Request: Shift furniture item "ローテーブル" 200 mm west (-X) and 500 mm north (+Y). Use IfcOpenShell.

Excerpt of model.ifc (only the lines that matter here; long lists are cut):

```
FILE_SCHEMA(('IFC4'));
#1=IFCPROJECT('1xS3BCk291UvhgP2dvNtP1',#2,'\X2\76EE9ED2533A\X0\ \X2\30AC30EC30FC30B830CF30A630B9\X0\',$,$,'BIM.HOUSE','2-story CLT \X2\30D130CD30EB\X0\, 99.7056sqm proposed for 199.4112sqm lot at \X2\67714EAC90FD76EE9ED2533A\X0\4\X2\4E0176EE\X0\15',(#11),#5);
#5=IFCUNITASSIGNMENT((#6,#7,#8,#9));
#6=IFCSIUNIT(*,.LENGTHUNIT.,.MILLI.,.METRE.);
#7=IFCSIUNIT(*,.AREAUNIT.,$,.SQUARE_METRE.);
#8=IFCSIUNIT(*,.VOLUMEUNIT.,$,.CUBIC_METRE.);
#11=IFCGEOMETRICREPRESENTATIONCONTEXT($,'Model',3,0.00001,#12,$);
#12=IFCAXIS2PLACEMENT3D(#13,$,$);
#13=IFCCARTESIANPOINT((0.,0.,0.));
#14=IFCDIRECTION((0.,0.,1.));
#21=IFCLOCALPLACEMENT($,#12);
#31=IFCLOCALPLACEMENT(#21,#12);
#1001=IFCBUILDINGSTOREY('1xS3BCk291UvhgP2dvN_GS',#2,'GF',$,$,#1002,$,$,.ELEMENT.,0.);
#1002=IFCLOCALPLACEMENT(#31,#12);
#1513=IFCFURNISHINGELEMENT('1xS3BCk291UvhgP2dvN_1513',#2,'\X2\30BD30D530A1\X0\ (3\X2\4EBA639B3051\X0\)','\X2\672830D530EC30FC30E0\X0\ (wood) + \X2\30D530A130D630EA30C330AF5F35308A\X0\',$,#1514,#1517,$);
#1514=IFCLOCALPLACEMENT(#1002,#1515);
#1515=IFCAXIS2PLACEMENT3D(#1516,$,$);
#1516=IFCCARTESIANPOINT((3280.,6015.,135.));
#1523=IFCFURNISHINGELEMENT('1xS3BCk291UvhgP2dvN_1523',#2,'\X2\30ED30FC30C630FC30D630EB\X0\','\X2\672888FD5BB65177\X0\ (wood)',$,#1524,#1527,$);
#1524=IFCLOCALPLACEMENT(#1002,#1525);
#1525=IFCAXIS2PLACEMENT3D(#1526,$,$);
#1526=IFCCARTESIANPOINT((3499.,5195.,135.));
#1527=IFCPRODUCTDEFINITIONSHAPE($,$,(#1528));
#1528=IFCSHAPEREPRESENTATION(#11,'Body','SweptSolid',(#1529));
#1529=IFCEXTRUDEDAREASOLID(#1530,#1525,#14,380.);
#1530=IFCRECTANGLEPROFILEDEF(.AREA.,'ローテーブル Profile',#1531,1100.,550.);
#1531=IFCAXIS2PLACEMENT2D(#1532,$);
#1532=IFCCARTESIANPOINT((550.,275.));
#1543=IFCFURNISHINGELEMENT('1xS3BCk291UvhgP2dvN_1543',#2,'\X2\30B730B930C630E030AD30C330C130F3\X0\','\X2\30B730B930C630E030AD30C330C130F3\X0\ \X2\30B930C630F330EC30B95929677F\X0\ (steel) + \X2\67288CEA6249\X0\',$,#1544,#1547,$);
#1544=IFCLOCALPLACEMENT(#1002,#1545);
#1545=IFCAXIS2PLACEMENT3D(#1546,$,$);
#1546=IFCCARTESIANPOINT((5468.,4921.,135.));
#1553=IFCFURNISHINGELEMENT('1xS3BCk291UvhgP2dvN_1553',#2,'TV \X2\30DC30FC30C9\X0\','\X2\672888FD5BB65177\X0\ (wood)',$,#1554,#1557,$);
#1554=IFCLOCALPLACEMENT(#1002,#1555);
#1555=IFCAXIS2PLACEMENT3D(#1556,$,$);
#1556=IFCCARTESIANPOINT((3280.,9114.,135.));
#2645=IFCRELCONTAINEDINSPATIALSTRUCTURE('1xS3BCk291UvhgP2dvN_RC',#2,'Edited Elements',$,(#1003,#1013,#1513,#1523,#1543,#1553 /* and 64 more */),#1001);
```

```python
import ifcopenshell
import ifcopenshell.api.geometry
import ifcopenshell.util.placement
import ifcopenshell.util.unit

model = ifcopenshell.open("model.ifc")
unit_scale = ifcopenshell.util.unit.calculate_unit_scale(model)

item = model.by_guid("1xS3BCk291UvhgP2dvN_1523")
matrix = ifcopenshell.util.placement.get_local_placement(item.ObjectPlacement)
matrix[0, 3] -= 0.2 / unit_scale
matrix[1, 3] += 0.5 / unit_scale
ifcopenshell.api.geometry.edit_object_placement(model, product=item, matrix=matrix, is_si=False)

print(ifcopenshell.util.placement.get_local_placement(item.ObjectPlacement).round(3) + 0.0)

model.write("model-out.ifc")
```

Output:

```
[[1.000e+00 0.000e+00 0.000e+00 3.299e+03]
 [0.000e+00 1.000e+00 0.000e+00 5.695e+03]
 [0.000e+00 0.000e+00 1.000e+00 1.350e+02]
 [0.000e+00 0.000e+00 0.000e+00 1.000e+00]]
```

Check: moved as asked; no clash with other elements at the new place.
